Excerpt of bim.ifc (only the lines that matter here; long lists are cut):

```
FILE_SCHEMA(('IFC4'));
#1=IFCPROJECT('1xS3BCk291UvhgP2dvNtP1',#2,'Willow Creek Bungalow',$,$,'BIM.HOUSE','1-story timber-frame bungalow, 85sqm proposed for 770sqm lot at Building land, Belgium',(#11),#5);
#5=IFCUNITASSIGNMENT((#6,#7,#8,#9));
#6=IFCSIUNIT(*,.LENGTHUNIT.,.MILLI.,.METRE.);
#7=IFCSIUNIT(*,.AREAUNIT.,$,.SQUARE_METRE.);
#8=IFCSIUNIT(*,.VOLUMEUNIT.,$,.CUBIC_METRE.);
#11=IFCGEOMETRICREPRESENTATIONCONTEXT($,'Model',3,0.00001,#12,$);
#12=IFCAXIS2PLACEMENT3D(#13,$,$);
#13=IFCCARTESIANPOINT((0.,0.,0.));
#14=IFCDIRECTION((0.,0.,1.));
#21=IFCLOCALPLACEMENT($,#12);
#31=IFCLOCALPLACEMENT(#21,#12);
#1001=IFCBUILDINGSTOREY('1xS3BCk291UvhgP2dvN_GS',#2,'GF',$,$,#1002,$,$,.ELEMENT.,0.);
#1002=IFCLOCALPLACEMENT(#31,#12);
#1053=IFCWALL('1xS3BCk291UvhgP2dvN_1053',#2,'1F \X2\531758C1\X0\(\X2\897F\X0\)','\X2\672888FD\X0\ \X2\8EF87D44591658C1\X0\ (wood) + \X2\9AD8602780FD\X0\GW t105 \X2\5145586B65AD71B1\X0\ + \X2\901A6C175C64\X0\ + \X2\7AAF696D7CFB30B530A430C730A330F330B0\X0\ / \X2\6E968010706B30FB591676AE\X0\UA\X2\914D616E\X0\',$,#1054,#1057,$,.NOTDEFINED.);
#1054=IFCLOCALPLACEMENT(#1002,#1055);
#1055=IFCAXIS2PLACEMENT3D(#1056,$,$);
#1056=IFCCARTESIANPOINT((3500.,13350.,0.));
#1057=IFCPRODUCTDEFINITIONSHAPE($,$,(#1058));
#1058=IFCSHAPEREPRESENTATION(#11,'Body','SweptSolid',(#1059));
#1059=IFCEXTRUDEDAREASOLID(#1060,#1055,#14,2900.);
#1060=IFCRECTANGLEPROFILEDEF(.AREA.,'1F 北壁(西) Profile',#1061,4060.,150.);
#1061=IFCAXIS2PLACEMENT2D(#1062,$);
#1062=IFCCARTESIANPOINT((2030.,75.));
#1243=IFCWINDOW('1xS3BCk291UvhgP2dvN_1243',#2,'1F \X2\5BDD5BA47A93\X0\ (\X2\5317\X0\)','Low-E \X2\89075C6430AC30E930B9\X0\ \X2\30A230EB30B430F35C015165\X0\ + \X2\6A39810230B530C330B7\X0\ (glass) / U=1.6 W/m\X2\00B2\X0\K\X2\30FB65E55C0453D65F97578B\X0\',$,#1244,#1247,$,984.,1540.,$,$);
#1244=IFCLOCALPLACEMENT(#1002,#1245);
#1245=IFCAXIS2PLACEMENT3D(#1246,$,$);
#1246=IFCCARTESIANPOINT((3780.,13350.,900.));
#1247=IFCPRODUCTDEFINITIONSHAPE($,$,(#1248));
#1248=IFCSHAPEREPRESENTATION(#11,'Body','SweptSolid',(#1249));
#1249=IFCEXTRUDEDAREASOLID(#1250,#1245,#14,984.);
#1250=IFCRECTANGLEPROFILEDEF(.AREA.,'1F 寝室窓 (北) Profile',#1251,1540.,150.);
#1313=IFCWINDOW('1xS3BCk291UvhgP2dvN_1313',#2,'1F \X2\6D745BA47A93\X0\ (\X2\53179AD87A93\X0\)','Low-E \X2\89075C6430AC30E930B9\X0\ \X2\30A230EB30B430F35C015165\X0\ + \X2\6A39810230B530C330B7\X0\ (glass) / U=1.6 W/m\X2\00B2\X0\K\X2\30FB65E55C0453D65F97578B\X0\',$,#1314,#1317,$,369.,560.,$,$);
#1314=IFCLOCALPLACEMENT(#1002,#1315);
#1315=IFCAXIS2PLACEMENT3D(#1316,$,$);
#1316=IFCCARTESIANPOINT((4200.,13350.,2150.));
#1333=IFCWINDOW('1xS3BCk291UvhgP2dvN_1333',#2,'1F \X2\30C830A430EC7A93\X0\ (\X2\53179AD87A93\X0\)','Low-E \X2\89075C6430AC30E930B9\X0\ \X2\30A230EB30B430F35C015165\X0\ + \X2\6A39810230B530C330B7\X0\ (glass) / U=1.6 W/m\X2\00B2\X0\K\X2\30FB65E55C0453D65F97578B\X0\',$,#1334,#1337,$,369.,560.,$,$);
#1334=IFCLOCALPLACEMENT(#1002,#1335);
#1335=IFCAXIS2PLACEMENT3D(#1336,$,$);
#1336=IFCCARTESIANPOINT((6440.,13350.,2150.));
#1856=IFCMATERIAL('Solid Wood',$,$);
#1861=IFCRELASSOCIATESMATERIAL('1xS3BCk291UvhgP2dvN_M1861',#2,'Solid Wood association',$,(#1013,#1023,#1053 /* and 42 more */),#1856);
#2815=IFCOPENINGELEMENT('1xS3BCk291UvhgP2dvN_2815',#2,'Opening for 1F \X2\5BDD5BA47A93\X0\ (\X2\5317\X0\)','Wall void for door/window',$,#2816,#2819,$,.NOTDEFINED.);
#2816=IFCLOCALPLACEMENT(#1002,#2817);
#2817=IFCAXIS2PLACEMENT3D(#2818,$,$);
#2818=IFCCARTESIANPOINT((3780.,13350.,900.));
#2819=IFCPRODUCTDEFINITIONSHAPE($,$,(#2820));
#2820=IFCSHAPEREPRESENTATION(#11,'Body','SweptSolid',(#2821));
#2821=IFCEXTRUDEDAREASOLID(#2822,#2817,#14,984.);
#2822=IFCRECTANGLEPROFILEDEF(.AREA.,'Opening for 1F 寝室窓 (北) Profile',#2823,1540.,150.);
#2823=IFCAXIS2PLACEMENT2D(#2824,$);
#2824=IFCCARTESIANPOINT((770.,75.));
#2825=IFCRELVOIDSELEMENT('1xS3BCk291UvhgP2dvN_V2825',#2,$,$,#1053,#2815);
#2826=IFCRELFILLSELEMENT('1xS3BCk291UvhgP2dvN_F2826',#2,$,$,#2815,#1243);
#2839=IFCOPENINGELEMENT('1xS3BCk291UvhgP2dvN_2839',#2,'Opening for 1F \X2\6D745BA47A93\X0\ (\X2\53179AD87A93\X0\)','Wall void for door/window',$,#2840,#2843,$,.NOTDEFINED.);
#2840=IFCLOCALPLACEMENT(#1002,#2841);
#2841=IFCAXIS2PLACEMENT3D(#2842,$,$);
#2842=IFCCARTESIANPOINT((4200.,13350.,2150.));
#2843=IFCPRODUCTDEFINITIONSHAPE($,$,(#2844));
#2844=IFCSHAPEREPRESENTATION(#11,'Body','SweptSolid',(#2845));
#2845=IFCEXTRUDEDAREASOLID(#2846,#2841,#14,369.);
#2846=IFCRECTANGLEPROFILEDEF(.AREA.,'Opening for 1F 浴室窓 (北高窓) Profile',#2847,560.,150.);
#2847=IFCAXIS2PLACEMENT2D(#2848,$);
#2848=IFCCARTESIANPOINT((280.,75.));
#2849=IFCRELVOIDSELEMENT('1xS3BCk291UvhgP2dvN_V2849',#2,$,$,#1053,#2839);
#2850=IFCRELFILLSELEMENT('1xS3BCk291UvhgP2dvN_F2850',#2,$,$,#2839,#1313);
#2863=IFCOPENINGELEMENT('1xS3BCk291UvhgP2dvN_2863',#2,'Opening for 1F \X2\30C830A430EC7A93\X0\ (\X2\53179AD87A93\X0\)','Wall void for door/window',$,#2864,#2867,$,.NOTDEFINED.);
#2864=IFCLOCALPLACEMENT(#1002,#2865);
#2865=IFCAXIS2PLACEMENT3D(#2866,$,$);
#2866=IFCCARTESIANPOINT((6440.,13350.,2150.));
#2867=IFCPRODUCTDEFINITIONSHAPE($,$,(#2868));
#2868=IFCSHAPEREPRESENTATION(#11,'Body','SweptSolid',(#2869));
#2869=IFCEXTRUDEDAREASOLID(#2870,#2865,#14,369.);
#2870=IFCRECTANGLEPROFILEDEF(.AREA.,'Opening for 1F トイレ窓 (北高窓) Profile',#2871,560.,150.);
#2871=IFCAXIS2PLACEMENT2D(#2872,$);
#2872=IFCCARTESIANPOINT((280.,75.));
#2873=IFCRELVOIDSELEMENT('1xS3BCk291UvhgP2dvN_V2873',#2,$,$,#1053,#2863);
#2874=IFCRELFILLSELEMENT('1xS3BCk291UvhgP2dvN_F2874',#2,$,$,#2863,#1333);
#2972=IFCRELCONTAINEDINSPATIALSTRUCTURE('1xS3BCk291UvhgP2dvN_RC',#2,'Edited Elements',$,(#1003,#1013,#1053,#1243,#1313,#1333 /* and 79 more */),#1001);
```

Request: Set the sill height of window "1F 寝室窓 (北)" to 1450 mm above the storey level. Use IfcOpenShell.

```python
import numpy as np
import ifcopenshell
import ifcopenshell.api.geometry
import ifcopenshell.geom
import ifcopenshell.util.element
import ifcopenshell.util.placement
import ifcopenshell.util.shape
import ifcopenshell.util.unit

model = ifcopenshell.open("bim.ifc")
unit_scale = ifcopenshell.util.unit.calculate_unit_scale(model)

window = model.by_guid("1xS3BCk291UvhgP2dvN_1243")
opening = window.FillsVoids[0].RelatingOpeningElement
storey = ifcopenshell.util.element.get_container(window, ifc_class="IfcBuildingStorey")
level = ifcopenshell.util.placement.get_local_placement(storey.ObjectPlacement)[2, 3]

# The opening's origin need not be at the sill, so measure its lowest point.
shape = ifcopenshell.geom.create_shape(ifcopenshell.geom.settings(), opening)
bottom = ifcopenshell.util.shape.get_shape_bottom_elevation(shape, shape.geometry) / unit_scale
dz = level + 1450.0 - bottom

shift = np.array([0.0, 0.0, dz])
# The window is not placed relative to its opening, so move both.
for product in (opening, window):
    matrix = ifcopenshell.util.placement.get_local_placement(product.ObjectPlacement)
    matrix[:3, 3] += shift
    ifcopenshell.api.geometry.edit_object_placement(model, product=product, matrix=matrix, is_si=False)

print(f"moved by {dz * unit_scale:+.3f} m")

model.write("bim_edited.ifc")
```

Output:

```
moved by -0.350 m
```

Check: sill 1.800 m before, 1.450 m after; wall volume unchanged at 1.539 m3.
